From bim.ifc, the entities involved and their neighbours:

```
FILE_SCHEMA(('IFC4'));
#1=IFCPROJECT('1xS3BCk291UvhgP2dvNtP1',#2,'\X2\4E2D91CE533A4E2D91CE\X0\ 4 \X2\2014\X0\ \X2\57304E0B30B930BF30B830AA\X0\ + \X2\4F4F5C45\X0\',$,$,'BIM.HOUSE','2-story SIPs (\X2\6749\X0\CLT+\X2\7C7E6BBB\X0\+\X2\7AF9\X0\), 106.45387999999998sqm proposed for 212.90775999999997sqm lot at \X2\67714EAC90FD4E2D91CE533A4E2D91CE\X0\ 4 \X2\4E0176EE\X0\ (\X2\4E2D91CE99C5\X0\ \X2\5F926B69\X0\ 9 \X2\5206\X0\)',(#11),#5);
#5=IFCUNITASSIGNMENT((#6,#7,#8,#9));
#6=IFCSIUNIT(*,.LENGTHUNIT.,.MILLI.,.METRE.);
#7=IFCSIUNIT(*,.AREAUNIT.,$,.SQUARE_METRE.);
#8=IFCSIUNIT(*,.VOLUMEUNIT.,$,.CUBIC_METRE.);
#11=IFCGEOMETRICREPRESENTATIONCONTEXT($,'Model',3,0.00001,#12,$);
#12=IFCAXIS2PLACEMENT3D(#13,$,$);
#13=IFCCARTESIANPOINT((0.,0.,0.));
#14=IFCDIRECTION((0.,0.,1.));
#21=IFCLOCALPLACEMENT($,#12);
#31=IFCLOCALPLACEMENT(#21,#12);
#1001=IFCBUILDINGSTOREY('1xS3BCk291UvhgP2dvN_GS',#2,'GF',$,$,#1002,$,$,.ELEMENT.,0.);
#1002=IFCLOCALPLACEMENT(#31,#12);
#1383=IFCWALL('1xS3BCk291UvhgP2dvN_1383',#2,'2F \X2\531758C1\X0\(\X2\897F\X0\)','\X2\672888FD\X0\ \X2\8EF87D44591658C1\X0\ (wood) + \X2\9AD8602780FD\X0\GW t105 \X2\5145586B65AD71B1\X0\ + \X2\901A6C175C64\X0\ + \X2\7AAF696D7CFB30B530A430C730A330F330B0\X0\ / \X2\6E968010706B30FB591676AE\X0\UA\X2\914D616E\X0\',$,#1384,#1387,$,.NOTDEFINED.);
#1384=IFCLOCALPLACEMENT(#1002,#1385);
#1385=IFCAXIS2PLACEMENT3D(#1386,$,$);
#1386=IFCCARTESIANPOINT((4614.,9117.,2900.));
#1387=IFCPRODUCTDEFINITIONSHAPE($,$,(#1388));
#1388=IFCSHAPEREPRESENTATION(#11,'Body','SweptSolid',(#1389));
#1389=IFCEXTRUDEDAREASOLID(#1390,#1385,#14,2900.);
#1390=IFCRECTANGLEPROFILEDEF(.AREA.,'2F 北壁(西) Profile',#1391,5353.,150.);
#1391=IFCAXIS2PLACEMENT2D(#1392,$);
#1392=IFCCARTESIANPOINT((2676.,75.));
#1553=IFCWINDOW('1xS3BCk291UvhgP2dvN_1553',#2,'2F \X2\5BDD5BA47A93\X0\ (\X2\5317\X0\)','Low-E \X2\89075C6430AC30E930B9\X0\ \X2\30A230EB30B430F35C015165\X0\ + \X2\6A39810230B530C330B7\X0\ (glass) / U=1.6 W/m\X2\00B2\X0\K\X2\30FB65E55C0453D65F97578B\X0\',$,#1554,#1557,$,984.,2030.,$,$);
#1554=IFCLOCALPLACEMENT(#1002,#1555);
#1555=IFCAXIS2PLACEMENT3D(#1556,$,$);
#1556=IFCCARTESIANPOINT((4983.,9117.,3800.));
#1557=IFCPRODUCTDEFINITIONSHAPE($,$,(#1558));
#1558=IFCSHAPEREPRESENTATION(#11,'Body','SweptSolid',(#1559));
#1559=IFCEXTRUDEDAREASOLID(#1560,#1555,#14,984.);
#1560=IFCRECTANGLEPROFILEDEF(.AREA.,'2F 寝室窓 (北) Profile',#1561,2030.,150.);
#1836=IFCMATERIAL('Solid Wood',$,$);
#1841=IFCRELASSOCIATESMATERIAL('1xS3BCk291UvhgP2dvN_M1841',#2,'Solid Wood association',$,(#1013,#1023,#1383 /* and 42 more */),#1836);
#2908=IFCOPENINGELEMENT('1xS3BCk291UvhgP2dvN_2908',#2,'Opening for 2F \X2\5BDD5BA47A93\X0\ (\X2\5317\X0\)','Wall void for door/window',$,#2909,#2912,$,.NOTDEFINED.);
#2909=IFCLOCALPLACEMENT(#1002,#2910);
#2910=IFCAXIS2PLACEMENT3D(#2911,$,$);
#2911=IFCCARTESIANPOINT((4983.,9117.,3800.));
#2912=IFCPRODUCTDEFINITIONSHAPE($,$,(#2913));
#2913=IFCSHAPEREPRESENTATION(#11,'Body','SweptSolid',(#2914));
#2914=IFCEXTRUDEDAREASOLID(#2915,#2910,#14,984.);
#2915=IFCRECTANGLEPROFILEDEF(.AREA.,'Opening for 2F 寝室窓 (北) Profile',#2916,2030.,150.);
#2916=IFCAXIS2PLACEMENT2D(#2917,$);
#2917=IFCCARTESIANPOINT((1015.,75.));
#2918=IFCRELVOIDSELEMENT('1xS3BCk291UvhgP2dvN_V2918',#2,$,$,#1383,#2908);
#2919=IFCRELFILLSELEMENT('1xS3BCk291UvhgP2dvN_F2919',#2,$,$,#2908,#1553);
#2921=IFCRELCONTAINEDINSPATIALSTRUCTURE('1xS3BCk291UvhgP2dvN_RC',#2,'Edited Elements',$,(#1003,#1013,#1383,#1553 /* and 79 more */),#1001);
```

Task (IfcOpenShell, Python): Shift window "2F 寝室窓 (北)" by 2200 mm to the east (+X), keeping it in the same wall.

```python
import ifcopenshell
import ifcopenshell.api.geometry
import ifcopenshell.util.placement
import ifcopenshell.util.unit

model = ifcopenshell.open("bim.ifc")
unit_scale = ifcopenshell.util.unit.calculate_unit_scale(model)

window = model.by_guid("1xS3BCk291UvhgP2dvN_1553")
opening = window.FillsVoids[0].RelatingOpeningElement
wall = opening.VoidsElements[0].RelatingBuildingElement

wall_matrix = ifcopenshell.util.placement.get_local_placement(wall.ObjectPlacement)
shift = wall_matrix[:3, 0] * 2.2 / unit_scale
before = ifcopenshell.util.placement.get_local_placement(window.ObjectPlacement)[:3, 3].copy()

# The window is not placed relative to its opening, so move both.
for product in (opening, window):
    matrix = ifcopenshell.util.placement.get_local_placement(product.ObjectPlacement)
    matrix[:3, 3] += shift
    ifcopenshell.api.geometry.edit_object_placement(model, product=product, matrix=matrix, is_si=False)

after = ifcopenshell.util.placement.get_local_placement(window.ObjectPlacement)[:3, 3]
print("window moved by", (after - before).round(3) + 0.0)

model.write("bim_edited.ifc")
```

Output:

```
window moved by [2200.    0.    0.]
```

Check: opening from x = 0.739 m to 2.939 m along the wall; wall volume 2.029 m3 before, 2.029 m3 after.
